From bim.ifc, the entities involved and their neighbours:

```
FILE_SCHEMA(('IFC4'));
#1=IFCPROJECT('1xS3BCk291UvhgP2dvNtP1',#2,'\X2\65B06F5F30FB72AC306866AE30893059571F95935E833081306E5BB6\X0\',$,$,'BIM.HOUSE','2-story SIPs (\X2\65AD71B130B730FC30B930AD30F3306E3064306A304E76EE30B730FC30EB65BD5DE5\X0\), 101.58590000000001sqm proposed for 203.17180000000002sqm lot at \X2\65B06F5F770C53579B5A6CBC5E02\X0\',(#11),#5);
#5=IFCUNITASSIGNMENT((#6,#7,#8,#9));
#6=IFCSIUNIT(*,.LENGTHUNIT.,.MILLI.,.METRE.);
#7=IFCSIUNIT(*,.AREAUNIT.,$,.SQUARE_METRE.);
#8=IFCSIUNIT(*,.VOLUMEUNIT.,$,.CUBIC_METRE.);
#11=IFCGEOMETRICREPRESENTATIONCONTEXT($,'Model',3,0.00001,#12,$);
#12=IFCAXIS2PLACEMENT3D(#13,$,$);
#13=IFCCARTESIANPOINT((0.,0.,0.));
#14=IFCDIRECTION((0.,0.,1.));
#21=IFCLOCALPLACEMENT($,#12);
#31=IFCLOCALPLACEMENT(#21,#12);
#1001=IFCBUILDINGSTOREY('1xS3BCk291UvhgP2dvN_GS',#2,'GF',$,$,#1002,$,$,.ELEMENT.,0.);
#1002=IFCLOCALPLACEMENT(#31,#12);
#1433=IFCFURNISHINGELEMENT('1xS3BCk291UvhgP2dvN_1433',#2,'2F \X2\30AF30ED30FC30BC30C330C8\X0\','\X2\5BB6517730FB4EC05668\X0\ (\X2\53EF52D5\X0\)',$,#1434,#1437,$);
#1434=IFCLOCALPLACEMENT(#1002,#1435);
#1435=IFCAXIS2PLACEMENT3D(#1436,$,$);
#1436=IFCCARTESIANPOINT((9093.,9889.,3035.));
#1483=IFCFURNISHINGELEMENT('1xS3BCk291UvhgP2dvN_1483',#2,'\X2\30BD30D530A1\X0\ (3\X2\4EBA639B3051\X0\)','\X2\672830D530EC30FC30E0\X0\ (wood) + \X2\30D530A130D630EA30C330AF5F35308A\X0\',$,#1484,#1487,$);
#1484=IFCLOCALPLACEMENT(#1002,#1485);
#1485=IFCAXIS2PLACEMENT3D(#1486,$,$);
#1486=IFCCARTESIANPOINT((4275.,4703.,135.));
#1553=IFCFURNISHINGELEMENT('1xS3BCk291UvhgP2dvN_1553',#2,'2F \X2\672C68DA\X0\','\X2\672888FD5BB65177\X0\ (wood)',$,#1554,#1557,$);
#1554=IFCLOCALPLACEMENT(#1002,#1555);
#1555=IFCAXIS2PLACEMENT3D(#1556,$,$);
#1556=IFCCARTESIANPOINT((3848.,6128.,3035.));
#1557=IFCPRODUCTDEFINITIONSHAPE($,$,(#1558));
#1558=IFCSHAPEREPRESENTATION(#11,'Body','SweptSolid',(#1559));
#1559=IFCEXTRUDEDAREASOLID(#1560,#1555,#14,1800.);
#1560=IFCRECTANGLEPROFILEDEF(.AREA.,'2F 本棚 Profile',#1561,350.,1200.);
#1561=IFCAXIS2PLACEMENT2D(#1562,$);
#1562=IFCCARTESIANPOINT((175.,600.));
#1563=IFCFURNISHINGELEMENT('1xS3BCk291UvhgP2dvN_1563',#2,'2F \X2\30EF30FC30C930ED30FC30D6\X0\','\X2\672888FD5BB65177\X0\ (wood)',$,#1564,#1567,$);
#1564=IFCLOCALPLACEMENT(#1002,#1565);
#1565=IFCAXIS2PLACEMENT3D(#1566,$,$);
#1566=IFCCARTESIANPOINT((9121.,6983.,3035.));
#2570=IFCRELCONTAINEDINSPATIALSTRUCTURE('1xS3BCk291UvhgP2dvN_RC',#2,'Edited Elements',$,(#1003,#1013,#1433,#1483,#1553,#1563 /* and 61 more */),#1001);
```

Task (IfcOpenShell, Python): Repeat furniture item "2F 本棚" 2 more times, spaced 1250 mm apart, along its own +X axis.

```python
import ifcopenshell
import ifcopenshell.api.geometry
import ifcopenshell.api.root
import ifcopenshell.util.element
import ifcopenshell.util.placement

model = ifcopenshell.open("bim.ifc")


def reuse_history(source, copy):
    """copy_class also copies each property set's owner history, people and application; keep the originals."""
    for rel in copy.IsDefinedBy:
        if rel.is_a("IfcRelDefinesByProperties") and (history := rel.RelatingPropertyDefinition.OwnerHistory):
            rel.RelatingPropertyDefinition.OwnerHistory = source.OwnerHistory
            ifcopenshell.util.element.remove_deep2(model, history)


source = model.by_guid("1xS3BCk291UvhgP2dvN_1553")
base = ifcopenshell.util.placement.get_local_placement(source.ObjectPlacement)
step = base[:3, 0] * 1250.0

for i in range(1, 3):
    copy = ifcopenshell.api.root.copy_class(model, product=source)
    copy.Representation = ifcopenshell.util.element.copy_deep(
        model, source.Representation, exclude=["IfcGeometricRepresentationContext", "IfcRepresentationMap"]
    )
    reuse_history(source, copy)
    matrix = base.copy()
    matrix[:3, 3] += i * step
    print("added at", matrix[:3, 3].round(3) + 0.0)
    ifcopenshell.api.geometry.edit_object_placement(model, product=copy, matrix=matrix, is_si=False)

model.write("bim_rev.ifc")
```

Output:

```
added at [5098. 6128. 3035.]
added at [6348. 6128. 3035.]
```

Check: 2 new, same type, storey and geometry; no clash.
